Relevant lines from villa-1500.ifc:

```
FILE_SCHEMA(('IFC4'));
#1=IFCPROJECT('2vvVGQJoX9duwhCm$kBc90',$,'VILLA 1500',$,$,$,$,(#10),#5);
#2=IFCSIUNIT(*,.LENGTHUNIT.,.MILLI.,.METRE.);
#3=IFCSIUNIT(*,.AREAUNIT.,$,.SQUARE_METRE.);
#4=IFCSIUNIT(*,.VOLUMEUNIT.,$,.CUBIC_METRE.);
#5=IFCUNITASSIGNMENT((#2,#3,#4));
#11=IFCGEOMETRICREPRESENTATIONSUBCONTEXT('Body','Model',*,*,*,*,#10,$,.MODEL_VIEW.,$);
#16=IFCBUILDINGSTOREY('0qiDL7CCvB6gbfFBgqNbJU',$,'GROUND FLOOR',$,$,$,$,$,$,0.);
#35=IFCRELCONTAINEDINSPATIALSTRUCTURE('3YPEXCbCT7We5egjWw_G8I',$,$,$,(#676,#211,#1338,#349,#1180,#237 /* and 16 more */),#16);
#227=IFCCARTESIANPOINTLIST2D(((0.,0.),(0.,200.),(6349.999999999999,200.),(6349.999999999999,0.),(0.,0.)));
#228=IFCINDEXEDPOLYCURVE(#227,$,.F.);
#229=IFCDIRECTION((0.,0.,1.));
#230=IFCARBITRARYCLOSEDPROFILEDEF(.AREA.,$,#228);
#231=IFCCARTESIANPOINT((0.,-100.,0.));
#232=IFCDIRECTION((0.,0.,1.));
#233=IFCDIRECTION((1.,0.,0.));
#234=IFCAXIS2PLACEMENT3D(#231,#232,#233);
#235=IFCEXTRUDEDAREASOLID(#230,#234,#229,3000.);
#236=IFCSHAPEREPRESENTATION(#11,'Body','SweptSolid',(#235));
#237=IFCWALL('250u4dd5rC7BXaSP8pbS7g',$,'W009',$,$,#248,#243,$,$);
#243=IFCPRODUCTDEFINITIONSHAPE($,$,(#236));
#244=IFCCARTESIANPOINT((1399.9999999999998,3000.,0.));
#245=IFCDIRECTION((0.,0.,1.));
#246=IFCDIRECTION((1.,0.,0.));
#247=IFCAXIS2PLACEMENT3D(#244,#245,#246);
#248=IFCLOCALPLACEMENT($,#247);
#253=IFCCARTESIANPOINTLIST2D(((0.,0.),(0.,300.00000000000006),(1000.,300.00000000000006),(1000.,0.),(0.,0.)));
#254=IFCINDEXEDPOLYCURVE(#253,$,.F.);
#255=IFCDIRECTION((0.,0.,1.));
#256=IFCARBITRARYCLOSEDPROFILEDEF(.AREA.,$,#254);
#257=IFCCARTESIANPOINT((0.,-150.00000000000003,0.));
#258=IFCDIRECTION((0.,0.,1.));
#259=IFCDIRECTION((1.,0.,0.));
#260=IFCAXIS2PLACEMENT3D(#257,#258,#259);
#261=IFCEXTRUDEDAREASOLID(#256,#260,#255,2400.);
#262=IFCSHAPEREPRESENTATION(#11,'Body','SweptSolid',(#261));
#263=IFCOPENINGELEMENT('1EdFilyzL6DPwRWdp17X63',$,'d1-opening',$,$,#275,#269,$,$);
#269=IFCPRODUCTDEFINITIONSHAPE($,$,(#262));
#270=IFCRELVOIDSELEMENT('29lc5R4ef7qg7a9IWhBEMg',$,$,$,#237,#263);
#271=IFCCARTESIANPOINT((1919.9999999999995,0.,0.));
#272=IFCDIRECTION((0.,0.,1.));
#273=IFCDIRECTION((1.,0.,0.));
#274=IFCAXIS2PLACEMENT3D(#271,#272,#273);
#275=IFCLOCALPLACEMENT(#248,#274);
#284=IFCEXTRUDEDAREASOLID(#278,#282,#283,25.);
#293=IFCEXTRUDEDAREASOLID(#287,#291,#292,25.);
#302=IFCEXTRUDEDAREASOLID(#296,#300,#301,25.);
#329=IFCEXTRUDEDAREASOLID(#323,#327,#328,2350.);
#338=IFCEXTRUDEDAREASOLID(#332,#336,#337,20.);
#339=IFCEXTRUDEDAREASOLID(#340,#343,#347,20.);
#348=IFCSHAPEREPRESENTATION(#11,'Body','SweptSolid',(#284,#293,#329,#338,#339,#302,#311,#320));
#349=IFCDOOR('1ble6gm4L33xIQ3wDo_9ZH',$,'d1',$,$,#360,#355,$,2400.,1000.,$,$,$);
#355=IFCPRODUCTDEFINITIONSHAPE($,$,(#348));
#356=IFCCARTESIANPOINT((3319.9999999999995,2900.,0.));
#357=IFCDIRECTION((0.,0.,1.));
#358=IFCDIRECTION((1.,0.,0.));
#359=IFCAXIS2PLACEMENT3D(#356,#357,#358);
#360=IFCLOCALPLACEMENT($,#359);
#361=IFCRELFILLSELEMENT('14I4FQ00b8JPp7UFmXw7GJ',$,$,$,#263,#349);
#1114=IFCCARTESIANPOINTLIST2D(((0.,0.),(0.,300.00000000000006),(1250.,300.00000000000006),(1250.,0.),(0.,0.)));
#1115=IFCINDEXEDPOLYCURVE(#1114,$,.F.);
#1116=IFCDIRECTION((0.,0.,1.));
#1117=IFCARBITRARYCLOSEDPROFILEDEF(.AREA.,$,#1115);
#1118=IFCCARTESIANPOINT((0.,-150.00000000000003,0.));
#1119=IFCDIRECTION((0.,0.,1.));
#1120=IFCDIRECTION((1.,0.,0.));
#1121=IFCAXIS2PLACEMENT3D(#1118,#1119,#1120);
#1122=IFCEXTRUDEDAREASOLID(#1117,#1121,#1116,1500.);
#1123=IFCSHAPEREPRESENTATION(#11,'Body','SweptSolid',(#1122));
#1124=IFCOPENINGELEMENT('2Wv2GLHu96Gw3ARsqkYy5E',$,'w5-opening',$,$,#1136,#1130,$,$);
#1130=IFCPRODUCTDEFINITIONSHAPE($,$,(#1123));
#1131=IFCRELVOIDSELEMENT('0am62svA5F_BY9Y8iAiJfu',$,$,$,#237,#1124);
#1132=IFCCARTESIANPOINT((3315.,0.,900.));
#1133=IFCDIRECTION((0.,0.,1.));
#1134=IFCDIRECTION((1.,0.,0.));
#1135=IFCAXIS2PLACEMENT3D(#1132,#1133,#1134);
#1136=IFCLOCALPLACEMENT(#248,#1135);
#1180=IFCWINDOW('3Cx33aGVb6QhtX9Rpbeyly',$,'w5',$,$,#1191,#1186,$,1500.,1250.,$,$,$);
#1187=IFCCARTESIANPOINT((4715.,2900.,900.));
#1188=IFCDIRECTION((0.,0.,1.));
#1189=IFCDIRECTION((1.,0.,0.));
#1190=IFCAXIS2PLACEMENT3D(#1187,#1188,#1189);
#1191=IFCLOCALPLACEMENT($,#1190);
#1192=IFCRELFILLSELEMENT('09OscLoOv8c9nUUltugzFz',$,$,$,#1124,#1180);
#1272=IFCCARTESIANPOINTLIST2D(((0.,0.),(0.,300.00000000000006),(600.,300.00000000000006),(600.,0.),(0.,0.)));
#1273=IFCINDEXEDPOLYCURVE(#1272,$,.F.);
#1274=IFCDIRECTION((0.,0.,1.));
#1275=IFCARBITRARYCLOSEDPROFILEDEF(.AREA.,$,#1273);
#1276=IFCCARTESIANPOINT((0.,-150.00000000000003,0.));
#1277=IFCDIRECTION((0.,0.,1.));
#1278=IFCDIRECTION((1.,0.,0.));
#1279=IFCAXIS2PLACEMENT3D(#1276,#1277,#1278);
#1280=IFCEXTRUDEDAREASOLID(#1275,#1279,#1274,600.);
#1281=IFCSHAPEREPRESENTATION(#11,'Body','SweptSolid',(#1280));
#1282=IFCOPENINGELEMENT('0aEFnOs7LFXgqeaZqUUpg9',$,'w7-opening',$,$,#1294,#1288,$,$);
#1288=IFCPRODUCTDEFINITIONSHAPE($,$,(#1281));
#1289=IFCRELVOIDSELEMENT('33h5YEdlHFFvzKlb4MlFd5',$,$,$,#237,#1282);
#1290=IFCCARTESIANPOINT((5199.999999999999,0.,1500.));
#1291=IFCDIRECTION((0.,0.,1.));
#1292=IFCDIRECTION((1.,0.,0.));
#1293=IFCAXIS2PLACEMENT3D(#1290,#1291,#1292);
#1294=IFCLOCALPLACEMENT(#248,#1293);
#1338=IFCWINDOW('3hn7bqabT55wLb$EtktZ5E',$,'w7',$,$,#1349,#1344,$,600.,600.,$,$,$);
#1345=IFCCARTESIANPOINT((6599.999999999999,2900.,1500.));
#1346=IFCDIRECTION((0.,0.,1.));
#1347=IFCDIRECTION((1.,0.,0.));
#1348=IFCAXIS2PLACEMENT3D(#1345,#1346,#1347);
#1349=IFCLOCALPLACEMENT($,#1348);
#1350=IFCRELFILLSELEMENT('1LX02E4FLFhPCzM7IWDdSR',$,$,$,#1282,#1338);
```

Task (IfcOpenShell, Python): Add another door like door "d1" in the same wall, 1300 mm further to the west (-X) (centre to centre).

```python
import ifcopenshell
import ifcopenshell.api.feature
import ifcopenshell.api.geometry
import ifcopenshell.api.root
import ifcopenshell.geom
import ifcopenshell.util.element
import ifcopenshell.util.placement
import ifcopenshell.util.shape
import ifcopenshell.util.unit

model = ifcopenshell.open("villa-1500.ifc")
unit_scale = ifcopenshell.util.unit.calculate_unit_scale(model)
settings = ifcopenshell.geom.settings()


def volume(element):
    """Net volume in cubic metres, openings subtracted."""
    shape = ifcopenshell.geom.create_shape(settings, element)
    return ifcopenshell.util.shape.get_volume(shape.geometry)


door = model.by_guid("1ble6gm4L33xIQ3wDo_9ZH")
opening = door.FillsVoids[0].RelatingOpeningElement
wall = opening.VoidsElements[0].RelatingBuildingElement
before = volume(wall)
shift = ifcopenshell.util.placement.get_local_placement(wall.ObjectPlacement)[:3, 0] * -1.3 / unit_scale

# copy_class copies the void relationship, type, container and properties, but no geometry.
new_opening = ifcopenshell.api.root.copy_class(model, product=opening)
new_opening.Representation = ifcopenshell.util.element.copy_deep(
    model, opening.Representation, exclude=["IfcGeometricRepresentationContext", "IfcRepresentationMap"]
)
new_door = ifcopenshell.api.root.copy_class(model, product=door)
new_door.Representation = ifcopenshell.util.element.copy_deep(
    model, door.Representation, exclude=["IfcGeometricRepresentationContext", "IfcRepresentationMap"]
)
ifcopenshell.api.feature.add_filling(model, opening=new_opening, element=new_door)

for old, new in ((opening, new_opening), (door, new_door)):
    matrix = ifcopenshell.util.placement.get_local_placement(old.ObjectPlacement)
    matrix[:3, 3] += shift
    ifcopenshell.api.geometry.edit_object_placement(model, product=new, matrix=matrix, is_si=False)

after = volume(wall)

print(f"wall volume {before:.3f} -> {after:.3f} m3")

model.write("villa-1500_updated.ifc")
```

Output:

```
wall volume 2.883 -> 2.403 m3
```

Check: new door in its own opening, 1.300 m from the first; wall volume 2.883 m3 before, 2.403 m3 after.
